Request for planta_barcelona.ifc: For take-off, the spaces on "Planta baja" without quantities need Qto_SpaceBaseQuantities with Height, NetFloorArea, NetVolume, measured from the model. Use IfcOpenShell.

First a look at what the model holds.

```python
import ifcopenshell
import ifcopenshell.util.element
import ifcopenshell.util.unit

model = ifcopenshell.open("planta_barcelona.ifc")
print(model.schema)
for unit_type in ("LENGTHUNIT", "AREAUNIT", "VOLUMEUNIT"):
    print(unit_type, ifcopenshell.util.unit.calculate_unit_scale(model, unit_type))
storey = next(s for s in model.by_type("IfcBuildingStorey") if s.Name == "Planta baja")
spaces = [e for e in ifcopenshell.util.element.get_decomposition(storey) if e.is_a("IfcSpace")]
for e in sorted(spaces, key=lambda e: e.id()):
    print(e.id(), e.is_a(), e.Name, list(ifcopenshell.util.element.get_psets(e, qtos_only=True)), sep=" | ")
```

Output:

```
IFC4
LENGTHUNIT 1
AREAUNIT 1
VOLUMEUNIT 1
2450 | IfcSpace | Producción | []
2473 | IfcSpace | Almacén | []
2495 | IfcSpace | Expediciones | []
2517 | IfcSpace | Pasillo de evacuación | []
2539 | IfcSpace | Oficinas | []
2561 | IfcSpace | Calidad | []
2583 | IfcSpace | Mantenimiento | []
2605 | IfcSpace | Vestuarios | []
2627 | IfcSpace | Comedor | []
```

```python
import ifcopenshell
import ifcopenshell.api.pset
import ifcopenshell.geom
import ifcopenshell.util.element
import ifcopenshell.util.shape
import ifcopenshell.util.unit

model = ifcopenshell.open("planta_barcelona.ifc")
unit_scale = ifcopenshell.util.unit.calculate_unit_scale(model)
area_scale = ifcopenshell.util.unit.calculate_unit_scale(model, "AREAUNIT")
volume_scale = ifcopenshell.util.unit.calculate_unit_scale(model, "VOLUMEUNIT")
settings = ifcopenshell.geom.settings()

storey = next(s for s in model.by_type("IfcBuildingStorey") if s.Name == "Planta baja")
spaces = [e for e in ifcopenshell.util.element.get_decomposition(storey) if e.is_a("IfcSpace")]

for e in sorted(spaces, key=lambda e: e.id()):
    if ifcopenshell.util.element.get_psets(e, qtos_only=True, should_inherit=False):
        continue
    # Geometry comes back in metres, in the element's own axes.
    shape = ifcopenshell.geom.create_shape(settings, e)
    values = {
        "Height": ifcopenshell.util.shape.get_z(shape.geometry) / unit_scale,
        "NetFloorArea": ifcopenshell.util.shape.get_footprint_area(shape.geometry) / area_scale,
        "NetVolume": ifcopenshell.util.shape.get_volume(shape.geometry) / volume_scale,
    }
    qto = ifcopenshell.api.pset.add_qto(model, product=e, name="Qto_SpaceBaseQuantities")
    ifcopenshell.api.pset.edit_qto(model, qto=qto, properties=values)
    print(e.id(), {k: round(v, 3) for k, v in values.items()})

model.write("planta_barcelona_updated.ifc")
```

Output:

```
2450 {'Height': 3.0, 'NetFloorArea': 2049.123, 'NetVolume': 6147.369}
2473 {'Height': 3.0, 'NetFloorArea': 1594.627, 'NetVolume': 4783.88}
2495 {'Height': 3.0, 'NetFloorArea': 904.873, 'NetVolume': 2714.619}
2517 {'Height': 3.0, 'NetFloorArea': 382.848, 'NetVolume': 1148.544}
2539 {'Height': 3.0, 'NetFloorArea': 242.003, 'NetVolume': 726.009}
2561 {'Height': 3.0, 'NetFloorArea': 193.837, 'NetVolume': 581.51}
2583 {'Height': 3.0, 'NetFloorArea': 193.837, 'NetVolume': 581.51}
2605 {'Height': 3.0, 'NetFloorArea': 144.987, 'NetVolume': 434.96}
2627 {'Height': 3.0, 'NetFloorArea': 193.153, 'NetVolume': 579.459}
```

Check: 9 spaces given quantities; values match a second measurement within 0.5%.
